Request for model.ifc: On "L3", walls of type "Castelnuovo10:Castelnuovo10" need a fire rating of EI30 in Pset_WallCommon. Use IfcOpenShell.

First a look at what the model holds.

```python
import ifcopenshell
import ifcopenshell.util.element

model = ifcopenshell.open("model.ifc")
print(model.schema)
storey = next(s for s in model.by_type("IfcBuildingStorey") if s.Name == "L3")
walls = [e for e in ifcopenshell.util.element.get_decomposition(storey) if e.is_a("IfcWall")]
seen = {}
for e in walls:
    element_type = ifcopenshell.util.element.get_type(e)
    key = (element_type.Name if element_type != e and element_type else None, ifcopenshell.util.element.get_pset(e, "Pset_WallCommon", "FireRating"))
    seen[key] = seen.get(key, 0) + 1
for (name, value), count in sorted(seen.items(), key=str):
    print(count, "x", name, "|", value)
```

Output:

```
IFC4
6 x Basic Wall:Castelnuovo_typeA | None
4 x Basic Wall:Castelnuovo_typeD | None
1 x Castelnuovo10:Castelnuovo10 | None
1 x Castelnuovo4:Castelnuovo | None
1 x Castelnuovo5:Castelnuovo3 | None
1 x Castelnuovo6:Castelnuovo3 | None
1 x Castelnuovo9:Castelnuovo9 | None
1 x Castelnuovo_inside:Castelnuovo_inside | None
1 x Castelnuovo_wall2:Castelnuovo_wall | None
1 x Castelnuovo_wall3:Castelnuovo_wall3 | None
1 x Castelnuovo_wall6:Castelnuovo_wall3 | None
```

```python
import ifcopenshell
import ifcopenshell.api.pset
import ifcopenshell.util.element

model = ifcopenshell.open("model.ifc")

storey = next(s for s in model.by_type("IfcBuildingStorey") if s.Name == "L3")
walls = [e for e in ifcopenshell.util.element.get_decomposition(storey) if e.is_a("IfcWall")]

count = 0
for e in walls:
    element_type = ifcopenshell.util.element.get_type(e)
    if element_type in (None, e) or element_type.Name != "Castelnuovo10:Castelnuovo10":
        continue
    # add_pset returns the element's existing set when there is one.
    pset = ifcopenshell.api.pset.add_pset(model, product=e, name="Pset_WallCommon")
    ifcopenshell.api.pset.edit_pset(model, pset=pset, properties={"FireRating": "EI30"})
    count += 1

print(count, "walls updated")

model.write("model_rev.ifc")
```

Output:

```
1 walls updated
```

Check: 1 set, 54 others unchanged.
